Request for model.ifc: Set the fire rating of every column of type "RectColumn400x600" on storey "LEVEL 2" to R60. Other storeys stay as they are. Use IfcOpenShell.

First a look at what the model holds.

```python
import ifcopenshell
import ifcopenshell.util.element

model = ifcopenshell.open("model.ifc")
print(model.schema)
storey = next(s for s in model.by_type("IfcBuildingStorey") if s.Name == "LEVEL 2")
columns = [e for e in ifcopenshell.util.element.get_decomposition(storey) if e.is_a("IfcColumn")]
seen = {}
for e in columns:
    element_type = ifcopenshell.util.element.get_type(e)
    key = (element_type.Name if element_type != e and element_type else None, ifcopenshell.util.element.get_pset(e, "Pset_ColumnCommon", "FireRating"))
    seen[key] = seen.get(key, 0) + 1
for (name, value), count in sorted(seen.items(), key=str):
    print(count, "x", name, "|", value)
```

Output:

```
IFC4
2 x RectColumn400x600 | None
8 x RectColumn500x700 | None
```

```python
import ifcopenshell
import ifcopenshell.api.pset
import ifcopenshell.util.element

model = ifcopenshell.open("model.ifc")

storey = next(s for s in model.by_type("IfcBuildingStorey") if s.Name == "LEVEL 2")
columns = [e for e in ifcopenshell.util.element.get_decomposition(storey) if e.is_a("IfcColumn")]

count = 0
for e in columns:
    element_type = ifcopenshell.util.element.get_type(e)
    if element_type in (None, e) or element_type.Name != "RectColumn400x600":
        continue
    # add_pset returns the element's existing set when there is one.
    pset = ifcopenshell.api.pset.add_pset(model, product=e, name="Pset_ColumnCommon")
    ifcopenshell.api.pset.edit_pset(model, pset=pset, properties={"FireRating": "R60"})
    count += 1

print(count, "columns updated")

model.write("model_v2.ifc")
```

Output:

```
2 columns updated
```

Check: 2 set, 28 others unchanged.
